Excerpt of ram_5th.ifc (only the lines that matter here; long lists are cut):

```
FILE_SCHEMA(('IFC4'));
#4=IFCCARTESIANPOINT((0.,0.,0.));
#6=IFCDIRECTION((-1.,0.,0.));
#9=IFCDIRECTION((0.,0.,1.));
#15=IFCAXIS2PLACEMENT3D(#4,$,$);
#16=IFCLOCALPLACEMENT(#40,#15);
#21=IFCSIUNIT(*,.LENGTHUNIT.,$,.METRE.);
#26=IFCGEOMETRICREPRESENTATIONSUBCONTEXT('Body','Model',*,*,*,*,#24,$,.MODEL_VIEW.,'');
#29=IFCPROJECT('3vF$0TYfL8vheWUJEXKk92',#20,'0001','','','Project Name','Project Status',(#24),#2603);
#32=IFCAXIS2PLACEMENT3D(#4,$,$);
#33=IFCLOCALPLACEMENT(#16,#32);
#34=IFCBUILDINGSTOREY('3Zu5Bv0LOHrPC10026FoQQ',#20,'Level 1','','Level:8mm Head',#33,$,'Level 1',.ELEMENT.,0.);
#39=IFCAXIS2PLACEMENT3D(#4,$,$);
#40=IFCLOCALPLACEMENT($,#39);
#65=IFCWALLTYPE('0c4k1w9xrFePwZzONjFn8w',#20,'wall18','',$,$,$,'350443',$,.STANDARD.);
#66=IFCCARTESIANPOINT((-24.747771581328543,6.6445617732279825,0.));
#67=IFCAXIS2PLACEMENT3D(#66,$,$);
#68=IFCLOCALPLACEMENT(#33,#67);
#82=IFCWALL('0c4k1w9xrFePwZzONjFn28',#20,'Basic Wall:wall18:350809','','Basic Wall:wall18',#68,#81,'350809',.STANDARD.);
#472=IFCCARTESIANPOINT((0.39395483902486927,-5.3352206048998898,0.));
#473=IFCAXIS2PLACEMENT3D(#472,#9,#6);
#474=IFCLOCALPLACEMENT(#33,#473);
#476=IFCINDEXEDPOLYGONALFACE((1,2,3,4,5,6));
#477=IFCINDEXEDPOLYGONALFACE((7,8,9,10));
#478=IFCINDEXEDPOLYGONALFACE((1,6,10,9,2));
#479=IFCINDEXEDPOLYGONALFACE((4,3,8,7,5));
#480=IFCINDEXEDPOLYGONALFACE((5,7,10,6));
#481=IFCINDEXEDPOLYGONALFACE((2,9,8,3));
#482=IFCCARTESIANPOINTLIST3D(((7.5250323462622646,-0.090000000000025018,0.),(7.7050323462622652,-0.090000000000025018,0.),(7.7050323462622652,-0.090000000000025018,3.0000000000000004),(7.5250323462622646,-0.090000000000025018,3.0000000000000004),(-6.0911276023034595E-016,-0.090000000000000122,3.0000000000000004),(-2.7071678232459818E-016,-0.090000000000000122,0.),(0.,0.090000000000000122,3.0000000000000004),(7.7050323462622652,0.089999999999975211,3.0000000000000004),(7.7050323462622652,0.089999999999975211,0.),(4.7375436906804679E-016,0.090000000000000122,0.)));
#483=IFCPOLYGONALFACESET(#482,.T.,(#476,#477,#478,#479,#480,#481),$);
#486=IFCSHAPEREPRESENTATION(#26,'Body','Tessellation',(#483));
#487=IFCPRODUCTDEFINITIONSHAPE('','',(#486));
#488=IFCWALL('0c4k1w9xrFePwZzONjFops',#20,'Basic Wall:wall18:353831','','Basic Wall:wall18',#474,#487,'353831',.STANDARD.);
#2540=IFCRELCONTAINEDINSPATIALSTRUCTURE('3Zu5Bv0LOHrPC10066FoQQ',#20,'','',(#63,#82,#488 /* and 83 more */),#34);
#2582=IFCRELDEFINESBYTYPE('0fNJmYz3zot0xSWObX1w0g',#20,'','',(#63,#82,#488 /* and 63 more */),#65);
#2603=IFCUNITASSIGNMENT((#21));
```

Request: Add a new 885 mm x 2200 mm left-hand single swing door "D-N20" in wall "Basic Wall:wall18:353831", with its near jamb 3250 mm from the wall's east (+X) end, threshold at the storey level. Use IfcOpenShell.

```python
import numpy as np
import ifcopenshell
import ifcopenshell.api.feature
import ifcopenshell.api.geometry
import ifcopenshell.api.root
import ifcopenshell.api.spatial
import ifcopenshell.geom
import ifcopenshell.util.element
import ifcopenshell.util.placement
import ifcopenshell.util.representation
import ifcopenshell.util.shape
import ifcopenshell.util.unit

model = ifcopenshell.open("ram_5th.ifc")
unit_scale = ifcopenshell.util.unit.calculate_unit_scale(model)
settings = ifcopenshell.geom.settings()


def volume(element):
    """Net volume in cubic metres, openings subtracted."""
    shape = ifcopenshell.geom.create_shape(settings, element)
    return ifcopenshell.util.shape.get_volume(shape.geometry)


wall = model.by_id(488)
storey = ifcopenshell.util.element.get_container(wall, ifc_class="IfcBuildingStorey")
context = ifcopenshell.util.representation.get_context(model, "Model", "Body", "MODEL_VIEW")
before = volume(wall)

width, height, from_end, sill = 0.885, 2.2, 3.25, 0.0  # metres

# The wall runs along its own X axis, and the end named is its -X end.
wall_shape = ifcopenshell.geom.create_shape(settings, wall)
x, y, z = ifcopenshell.util.shape.get_vertices(wall_shape.geometry).T
start = x.min() + from_end
face, thickness = float(y.min()), float(y.max() - y.min())
wall_matrix = ifcopenshell.util.placement.get_local_placement(wall.ObjectPlacement)
level = ifcopenshell.util.placement.get_local_placement(storey.ObjectPlacement)[2, 3]


def in_wall(x, y):
    """Placement at x, y metres in the wall's axes, at sill height."""
    matrix = wall_matrix.copy()
    matrix[:, 3] = wall_matrix @ np.array([x / unit_scale, y / unit_scale, 0.0, 1.0])
    matrix[2, 3] = level + sill / unit_scale
    return matrix


# Opening: a box that overshoots both wall faces by 50 mm.
opening = ifcopenshell.api.root.create_entity(model, ifc_class="IfcOpeningElement", predefined_type="OPENING")
box = ifcopenshell.api.geometry.add_wall_representation(
    model, context=context, length=width, height=height, thickness=thickness + 0.1
)
ifcopenshell.api.geometry.assign_representation(model, product=opening, representation=box)
ifcopenshell.api.geometry.edit_object_placement(model, product=opening, matrix=in_wall(start, face - 0.05), is_si=False)
ifcopenshell.api.feature.add_feature(model, feature=opening, element=wall)

door = ifcopenshell.api.root.create_entity(model, ifc_class="IfcDoor", name="D-N20", predefined_type="DOOR")
door.OverallWidth, door.OverallHeight = width / unit_scale, height / unit_scale
door.OperationType = "SINGLE_SWING_LEFT"
body = ifcopenshell.api.geometry.add_door_representation(
    model,
    context=context,
    overall_width=door.OverallWidth,
    overall_height=door.OverallHeight,
    operation_type="SINGLE_SWING_LEFT",
    lining_properties={"LiningDepth": thickness / unit_scale, "ThresholdDepth": thickness / unit_scale},
)
ifcopenshell.api.geometry.assign_representation(model, product=door, representation=body)
ifcopenshell.api.spatial.assign_container(model, products=[door], relating_structure=storey)
ifcopenshell.api.feature.add_filling(model, opening=opening, element=door)

# The lining spans the wall, so the door starts at the wall face.
ifcopenshell.api.geometry.edit_object_placement(model, product=door, matrix=in_wall(start, face), is_si=False)

after = volume(wall)

print(f"wall volume {before:.3f} -> {after:.3f} m3")

model.write("ram_5th-out.ifc")
```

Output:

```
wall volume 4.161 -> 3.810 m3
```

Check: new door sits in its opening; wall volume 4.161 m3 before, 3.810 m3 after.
